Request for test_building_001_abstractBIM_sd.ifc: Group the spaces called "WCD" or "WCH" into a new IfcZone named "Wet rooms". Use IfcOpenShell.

First a look at what the model holds.

```python
import ifcopenshell

model = ifcopenshell.open("test_building_001_abstractBIM_sd.ifc")
print(model.schema)
seen = {}
for space in model.by_type("IfcSpace"):
    seen[space.LongName] = seen.get(space.LongName, 0) + 1
for name, count in sorted(seen.items(), key=str):
    print(count, "x", name)
print("zones:", [z.Name for z in model.by_type("IfcZone")][:20])
```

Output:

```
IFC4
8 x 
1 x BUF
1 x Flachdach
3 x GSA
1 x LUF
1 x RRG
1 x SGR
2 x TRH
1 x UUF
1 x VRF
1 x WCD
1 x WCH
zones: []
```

```python
import ifcopenshell
import ifcopenshell.api.group
import ifcopenshell.api.root

model = ifcopenshell.open("test_building_001_abstractBIM_sd.ifc")

names = {"WCD", "WCH"}
spaces = [s for s in model.by_type("IfcSpace") if s.LongName in names]

zone = ifcopenshell.api.root.create_entity(model, ifc_class="IfcZone", name="Wet rooms")
ifcopenshell.api.group.assign_group(model, products=spaces, group=zone)
print(len(spaces), "spaces in", zone.Name)

model.write("test_building_001_abstractBIM_sd_updated.ifc")
```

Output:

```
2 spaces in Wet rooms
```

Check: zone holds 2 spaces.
